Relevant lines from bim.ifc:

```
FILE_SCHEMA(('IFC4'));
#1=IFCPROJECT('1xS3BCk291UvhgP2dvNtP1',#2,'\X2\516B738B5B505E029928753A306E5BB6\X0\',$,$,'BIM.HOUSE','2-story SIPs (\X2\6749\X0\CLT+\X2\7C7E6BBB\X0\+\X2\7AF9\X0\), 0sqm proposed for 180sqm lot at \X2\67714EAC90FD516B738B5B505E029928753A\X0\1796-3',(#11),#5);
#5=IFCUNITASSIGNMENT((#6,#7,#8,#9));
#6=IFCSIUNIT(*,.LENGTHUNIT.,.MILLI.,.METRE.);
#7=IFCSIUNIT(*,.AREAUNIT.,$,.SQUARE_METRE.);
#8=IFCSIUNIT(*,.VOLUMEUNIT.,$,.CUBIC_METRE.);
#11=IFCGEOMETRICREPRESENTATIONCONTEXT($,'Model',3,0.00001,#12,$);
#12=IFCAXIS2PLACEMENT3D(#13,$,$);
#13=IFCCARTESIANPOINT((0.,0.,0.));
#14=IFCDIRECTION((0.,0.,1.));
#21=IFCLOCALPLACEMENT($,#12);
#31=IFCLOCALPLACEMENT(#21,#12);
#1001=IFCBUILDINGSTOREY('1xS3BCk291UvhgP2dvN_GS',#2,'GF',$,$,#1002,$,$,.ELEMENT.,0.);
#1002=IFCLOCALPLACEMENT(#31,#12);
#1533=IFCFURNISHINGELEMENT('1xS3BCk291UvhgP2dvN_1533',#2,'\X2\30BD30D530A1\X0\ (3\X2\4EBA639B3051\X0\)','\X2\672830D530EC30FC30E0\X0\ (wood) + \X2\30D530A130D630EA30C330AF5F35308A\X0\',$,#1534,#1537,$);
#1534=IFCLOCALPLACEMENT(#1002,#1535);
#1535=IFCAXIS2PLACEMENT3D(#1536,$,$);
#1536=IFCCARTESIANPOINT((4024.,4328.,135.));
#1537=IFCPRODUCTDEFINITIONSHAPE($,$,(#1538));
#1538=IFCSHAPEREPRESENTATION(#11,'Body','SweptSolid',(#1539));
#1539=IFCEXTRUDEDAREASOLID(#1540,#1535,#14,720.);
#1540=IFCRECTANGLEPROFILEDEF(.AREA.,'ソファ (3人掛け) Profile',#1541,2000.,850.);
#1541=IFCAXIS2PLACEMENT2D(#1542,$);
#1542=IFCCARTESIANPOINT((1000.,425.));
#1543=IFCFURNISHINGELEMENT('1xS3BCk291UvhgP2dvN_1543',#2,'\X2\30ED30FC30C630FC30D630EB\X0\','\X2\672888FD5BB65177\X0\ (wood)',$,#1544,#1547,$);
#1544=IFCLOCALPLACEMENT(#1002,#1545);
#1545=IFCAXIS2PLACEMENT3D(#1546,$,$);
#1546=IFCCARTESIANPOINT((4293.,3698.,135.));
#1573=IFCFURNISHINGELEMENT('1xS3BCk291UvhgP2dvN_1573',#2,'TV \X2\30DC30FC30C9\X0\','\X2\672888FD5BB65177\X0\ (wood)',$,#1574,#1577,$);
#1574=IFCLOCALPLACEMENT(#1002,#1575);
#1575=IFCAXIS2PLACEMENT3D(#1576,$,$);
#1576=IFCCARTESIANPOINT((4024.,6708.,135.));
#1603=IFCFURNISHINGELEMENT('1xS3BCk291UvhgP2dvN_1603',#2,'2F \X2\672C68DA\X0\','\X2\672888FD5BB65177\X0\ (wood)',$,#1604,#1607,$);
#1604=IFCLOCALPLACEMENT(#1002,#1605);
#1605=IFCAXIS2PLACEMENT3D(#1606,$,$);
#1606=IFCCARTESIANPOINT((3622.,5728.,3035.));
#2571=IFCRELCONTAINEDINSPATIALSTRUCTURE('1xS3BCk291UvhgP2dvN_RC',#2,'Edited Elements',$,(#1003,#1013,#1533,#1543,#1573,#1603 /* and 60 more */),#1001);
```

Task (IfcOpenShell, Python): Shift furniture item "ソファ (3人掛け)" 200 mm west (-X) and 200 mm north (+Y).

```python
import ifcopenshell
import ifcopenshell.api.geometry
import ifcopenshell.util.placement

model = ifcopenshell.open("bim.ifc")

item = model.by_guid("1xS3BCk291UvhgP2dvN_1533")
matrix = ifcopenshell.util.placement.get_local_placement(item.ObjectPlacement)
matrix[0, 3] -= 200.0
matrix[1, 3] += 200.0
ifcopenshell.api.geometry.edit_object_placement(model, product=item, matrix=matrix, is_si=False)

print(ifcopenshell.util.placement.get_local_placement(item.ObjectPlacement).round(3) + 0.0)

model.write("bim_edited.ifc")
```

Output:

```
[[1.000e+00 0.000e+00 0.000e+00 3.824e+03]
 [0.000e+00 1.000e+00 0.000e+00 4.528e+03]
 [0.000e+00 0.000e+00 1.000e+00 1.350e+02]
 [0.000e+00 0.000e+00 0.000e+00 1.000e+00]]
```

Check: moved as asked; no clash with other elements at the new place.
